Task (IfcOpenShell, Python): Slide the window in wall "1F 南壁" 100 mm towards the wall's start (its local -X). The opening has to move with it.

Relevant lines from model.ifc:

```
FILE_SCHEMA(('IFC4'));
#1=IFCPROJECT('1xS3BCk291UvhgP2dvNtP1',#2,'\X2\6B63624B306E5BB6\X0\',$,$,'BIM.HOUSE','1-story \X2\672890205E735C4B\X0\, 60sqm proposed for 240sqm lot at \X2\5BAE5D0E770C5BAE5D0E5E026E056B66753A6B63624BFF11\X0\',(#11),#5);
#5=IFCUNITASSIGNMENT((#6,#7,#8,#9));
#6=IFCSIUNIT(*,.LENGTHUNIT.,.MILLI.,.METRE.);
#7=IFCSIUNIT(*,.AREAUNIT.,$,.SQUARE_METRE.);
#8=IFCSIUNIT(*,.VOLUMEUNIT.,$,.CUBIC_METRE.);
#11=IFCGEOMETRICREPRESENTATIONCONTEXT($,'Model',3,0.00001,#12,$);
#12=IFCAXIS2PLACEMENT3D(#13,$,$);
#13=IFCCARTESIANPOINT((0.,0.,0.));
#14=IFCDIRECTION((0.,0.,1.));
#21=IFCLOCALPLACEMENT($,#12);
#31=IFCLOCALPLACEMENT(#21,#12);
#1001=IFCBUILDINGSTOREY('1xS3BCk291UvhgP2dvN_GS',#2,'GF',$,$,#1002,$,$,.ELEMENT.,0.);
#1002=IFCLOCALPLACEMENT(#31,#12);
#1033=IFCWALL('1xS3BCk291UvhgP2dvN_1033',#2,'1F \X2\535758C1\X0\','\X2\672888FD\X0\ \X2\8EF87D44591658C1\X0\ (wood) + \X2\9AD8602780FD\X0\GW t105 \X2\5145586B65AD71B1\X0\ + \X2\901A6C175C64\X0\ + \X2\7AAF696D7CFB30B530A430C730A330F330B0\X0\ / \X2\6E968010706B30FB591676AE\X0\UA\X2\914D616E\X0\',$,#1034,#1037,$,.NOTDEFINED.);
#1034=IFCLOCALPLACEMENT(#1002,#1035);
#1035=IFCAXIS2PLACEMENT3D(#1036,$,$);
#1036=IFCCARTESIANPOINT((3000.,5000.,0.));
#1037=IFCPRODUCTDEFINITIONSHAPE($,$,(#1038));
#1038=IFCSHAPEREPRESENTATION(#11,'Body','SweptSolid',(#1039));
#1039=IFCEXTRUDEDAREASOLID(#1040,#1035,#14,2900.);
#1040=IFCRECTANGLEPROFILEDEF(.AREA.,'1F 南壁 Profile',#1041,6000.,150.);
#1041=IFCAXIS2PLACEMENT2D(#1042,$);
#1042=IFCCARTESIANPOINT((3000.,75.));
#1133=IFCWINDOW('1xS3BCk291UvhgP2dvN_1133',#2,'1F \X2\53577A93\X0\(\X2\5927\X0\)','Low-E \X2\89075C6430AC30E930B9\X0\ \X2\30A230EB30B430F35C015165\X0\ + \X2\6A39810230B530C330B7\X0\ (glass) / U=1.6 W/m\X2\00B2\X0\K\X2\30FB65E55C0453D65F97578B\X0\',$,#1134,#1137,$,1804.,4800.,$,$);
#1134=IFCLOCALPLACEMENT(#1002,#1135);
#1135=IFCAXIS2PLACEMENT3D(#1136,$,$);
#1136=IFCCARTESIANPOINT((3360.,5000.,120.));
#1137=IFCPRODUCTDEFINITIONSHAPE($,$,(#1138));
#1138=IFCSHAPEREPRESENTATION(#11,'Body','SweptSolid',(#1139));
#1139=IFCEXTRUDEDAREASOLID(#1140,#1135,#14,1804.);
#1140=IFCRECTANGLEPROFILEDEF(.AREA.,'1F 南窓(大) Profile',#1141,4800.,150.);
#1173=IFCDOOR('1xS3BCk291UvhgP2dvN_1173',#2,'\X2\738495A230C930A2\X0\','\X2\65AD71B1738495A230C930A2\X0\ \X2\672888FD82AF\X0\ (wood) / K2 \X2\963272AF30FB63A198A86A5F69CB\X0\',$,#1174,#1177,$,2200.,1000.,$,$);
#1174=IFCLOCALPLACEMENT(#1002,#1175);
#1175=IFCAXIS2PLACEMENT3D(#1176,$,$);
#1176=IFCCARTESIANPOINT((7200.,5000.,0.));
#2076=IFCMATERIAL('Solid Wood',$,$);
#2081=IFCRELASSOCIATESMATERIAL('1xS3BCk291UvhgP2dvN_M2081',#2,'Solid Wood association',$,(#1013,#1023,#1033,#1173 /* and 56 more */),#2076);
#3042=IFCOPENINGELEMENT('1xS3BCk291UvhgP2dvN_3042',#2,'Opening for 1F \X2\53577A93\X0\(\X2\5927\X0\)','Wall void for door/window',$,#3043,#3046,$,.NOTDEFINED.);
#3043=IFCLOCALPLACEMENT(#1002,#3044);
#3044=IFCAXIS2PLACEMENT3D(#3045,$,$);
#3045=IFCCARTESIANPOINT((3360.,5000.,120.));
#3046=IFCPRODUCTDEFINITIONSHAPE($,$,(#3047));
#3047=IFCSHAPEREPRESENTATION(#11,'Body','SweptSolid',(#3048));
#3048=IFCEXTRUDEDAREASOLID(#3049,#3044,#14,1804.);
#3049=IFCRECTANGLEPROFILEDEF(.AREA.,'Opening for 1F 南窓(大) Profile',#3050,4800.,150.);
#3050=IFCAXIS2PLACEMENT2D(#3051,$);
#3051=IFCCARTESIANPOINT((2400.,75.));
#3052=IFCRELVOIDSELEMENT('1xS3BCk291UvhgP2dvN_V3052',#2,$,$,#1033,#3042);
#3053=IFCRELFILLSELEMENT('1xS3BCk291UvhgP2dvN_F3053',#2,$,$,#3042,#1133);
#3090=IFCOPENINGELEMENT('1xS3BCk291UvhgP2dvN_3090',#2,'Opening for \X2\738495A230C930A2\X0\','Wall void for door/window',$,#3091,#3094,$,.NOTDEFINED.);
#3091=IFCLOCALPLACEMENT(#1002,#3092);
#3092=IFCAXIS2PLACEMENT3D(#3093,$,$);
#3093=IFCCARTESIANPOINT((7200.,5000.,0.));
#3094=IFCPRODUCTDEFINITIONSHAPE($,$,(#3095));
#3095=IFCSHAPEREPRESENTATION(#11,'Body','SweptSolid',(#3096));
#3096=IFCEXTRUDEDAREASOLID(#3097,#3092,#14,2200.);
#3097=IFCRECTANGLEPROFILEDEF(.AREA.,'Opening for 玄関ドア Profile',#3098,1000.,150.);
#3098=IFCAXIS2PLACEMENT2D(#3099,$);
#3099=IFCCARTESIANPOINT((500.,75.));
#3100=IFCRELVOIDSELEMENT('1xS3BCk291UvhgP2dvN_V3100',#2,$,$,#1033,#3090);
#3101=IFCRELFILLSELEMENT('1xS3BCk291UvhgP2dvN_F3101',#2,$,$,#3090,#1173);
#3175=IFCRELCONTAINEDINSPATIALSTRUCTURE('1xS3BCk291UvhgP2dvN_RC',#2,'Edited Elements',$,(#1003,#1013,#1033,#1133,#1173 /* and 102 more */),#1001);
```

```python
import ifcopenshell
import ifcopenshell.api.geometry
import ifcopenshell.util.placement
import ifcopenshell.util.unit

model = ifcopenshell.open("model.ifc")
unit_scale = ifcopenshell.util.unit.calculate_unit_scale(model)

window = model.by_guid("1xS3BCk291UvhgP2dvN_1133")
opening = window.FillsVoids[0].RelatingOpeningElement
wall = opening.VoidsElements[0].RelatingBuildingElement

wall_matrix = ifcopenshell.util.placement.get_local_placement(wall.ObjectPlacement)
shift = wall_matrix[:3, 0] * -0.1 / unit_scale
before = ifcopenshell.util.placement.get_local_placement(window.ObjectPlacement)[:3, 3].copy()

# The window is not placed relative to its opening, so move both.
for product in (opening, window):
    matrix = ifcopenshell.util.placement.get_local_placement(product.ObjectPlacement)
    matrix[:3, 3] += shift
    ifcopenshell.api.geometry.edit_object_placement(model, product=product, matrix=matrix, is_si=False)

after = ifcopenshell.util.placement.get_local_placement(window.ObjectPlacement)[:3, 3]
print("window moved by", (after - before).round(3) + 0.0)

model.write("model_updated.ifc")
```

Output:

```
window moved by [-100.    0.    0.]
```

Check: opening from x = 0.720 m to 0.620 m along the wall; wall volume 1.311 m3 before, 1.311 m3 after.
